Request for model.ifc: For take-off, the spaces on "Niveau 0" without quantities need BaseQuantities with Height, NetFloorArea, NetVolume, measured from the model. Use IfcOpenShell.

First a look at what the model holds.

```python
import ifcopenshell
import ifcopenshell.util.element
import ifcopenshell.util.unit

model = ifcopenshell.open("model.ifc")
print(model.schema)
for unit_type in ("LENGTHUNIT", "AREAUNIT", "VOLUMEUNIT"):
    print(unit_type, ifcopenshell.util.unit.calculate_unit_scale(model, unit_type))
storey = next(s for s in model.by_type("IfcBuildingStorey") if s.Name == "Niveau 0")
spaces = [e for e in ifcopenshell.util.element.get_decomposition(storey) if e.is_a("IfcSpace")]
for e in sorted(spaces, key=lambda e: e.id()):
    print(e.id(), e.is_a(), e.Name, list(ifcopenshell.util.element.get_psets(e, qtos_only=True)), sep=" | ")
```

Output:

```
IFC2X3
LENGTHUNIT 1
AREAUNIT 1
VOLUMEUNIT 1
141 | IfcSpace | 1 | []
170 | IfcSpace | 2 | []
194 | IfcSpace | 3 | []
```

```python
import ifcopenshell
import ifcopenshell.api.pset
import ifcopenshell.geom
import ifcopenshell.util.element
import ifcopenshell.util.shape
import ifcopenshell.util.unit

model = ifcopenshell.open("model.ifc")
unit_scale = ifcopenshell.util.unit.calculate_unit_scale(model)
area_scale = ifcopenshell.util.unit.calculate_unit_scale(model, "AREAUNIT")
volume_scale = ifcopenshell.util.unit.calculate_unit_scale(model, "VOLUMEUNIT")
settings = ifcopenshell.geom.settings()

storey = next(s for s in model.by_type("IfcBuildingStorey") if s.Name == "Niveau 0")
spaces = [e for e in ifcopenshell.util.element.get_decomposition(storey) if e.is_a("IfcSpace")]

for e in sorted(spaces, key=lambda e: e.id()):
    if ifcopenshell.util.element.get_psets(e, qtos_only=True, should_inherit=False):
        continue
    # Geometry comes back in metres, in the element's own axes.
    shape = ifcopenshell.geom.create_shape(settings, e)
    values = {
        "Height": ifcopenshell.util.shape.get_z(shape.geometry) / unit_scale,
        "NetFloorArea": ifcopenshell.util.shape.get_footprint_area(shape.geometry) / area_scale,
        "NetVolume": ifcopenshell.util.shape.get_volume(shape.geometry) / volume_scale,
    }
    qto = ifcopenshell.api.pset.add_qto(model, product=e, name="BaseQuantities")
    ifcopenshell.api.pset.edit_qto(model, qto=qto, properties=values)
    print(e.id(), {k: round(v, 3) for k, v in values.items()})

model.write("model_v2.ifc")
```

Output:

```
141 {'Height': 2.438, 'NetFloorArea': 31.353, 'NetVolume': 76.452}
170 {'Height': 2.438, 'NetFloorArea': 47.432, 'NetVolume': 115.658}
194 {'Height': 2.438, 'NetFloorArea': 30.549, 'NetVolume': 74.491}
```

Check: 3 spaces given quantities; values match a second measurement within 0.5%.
